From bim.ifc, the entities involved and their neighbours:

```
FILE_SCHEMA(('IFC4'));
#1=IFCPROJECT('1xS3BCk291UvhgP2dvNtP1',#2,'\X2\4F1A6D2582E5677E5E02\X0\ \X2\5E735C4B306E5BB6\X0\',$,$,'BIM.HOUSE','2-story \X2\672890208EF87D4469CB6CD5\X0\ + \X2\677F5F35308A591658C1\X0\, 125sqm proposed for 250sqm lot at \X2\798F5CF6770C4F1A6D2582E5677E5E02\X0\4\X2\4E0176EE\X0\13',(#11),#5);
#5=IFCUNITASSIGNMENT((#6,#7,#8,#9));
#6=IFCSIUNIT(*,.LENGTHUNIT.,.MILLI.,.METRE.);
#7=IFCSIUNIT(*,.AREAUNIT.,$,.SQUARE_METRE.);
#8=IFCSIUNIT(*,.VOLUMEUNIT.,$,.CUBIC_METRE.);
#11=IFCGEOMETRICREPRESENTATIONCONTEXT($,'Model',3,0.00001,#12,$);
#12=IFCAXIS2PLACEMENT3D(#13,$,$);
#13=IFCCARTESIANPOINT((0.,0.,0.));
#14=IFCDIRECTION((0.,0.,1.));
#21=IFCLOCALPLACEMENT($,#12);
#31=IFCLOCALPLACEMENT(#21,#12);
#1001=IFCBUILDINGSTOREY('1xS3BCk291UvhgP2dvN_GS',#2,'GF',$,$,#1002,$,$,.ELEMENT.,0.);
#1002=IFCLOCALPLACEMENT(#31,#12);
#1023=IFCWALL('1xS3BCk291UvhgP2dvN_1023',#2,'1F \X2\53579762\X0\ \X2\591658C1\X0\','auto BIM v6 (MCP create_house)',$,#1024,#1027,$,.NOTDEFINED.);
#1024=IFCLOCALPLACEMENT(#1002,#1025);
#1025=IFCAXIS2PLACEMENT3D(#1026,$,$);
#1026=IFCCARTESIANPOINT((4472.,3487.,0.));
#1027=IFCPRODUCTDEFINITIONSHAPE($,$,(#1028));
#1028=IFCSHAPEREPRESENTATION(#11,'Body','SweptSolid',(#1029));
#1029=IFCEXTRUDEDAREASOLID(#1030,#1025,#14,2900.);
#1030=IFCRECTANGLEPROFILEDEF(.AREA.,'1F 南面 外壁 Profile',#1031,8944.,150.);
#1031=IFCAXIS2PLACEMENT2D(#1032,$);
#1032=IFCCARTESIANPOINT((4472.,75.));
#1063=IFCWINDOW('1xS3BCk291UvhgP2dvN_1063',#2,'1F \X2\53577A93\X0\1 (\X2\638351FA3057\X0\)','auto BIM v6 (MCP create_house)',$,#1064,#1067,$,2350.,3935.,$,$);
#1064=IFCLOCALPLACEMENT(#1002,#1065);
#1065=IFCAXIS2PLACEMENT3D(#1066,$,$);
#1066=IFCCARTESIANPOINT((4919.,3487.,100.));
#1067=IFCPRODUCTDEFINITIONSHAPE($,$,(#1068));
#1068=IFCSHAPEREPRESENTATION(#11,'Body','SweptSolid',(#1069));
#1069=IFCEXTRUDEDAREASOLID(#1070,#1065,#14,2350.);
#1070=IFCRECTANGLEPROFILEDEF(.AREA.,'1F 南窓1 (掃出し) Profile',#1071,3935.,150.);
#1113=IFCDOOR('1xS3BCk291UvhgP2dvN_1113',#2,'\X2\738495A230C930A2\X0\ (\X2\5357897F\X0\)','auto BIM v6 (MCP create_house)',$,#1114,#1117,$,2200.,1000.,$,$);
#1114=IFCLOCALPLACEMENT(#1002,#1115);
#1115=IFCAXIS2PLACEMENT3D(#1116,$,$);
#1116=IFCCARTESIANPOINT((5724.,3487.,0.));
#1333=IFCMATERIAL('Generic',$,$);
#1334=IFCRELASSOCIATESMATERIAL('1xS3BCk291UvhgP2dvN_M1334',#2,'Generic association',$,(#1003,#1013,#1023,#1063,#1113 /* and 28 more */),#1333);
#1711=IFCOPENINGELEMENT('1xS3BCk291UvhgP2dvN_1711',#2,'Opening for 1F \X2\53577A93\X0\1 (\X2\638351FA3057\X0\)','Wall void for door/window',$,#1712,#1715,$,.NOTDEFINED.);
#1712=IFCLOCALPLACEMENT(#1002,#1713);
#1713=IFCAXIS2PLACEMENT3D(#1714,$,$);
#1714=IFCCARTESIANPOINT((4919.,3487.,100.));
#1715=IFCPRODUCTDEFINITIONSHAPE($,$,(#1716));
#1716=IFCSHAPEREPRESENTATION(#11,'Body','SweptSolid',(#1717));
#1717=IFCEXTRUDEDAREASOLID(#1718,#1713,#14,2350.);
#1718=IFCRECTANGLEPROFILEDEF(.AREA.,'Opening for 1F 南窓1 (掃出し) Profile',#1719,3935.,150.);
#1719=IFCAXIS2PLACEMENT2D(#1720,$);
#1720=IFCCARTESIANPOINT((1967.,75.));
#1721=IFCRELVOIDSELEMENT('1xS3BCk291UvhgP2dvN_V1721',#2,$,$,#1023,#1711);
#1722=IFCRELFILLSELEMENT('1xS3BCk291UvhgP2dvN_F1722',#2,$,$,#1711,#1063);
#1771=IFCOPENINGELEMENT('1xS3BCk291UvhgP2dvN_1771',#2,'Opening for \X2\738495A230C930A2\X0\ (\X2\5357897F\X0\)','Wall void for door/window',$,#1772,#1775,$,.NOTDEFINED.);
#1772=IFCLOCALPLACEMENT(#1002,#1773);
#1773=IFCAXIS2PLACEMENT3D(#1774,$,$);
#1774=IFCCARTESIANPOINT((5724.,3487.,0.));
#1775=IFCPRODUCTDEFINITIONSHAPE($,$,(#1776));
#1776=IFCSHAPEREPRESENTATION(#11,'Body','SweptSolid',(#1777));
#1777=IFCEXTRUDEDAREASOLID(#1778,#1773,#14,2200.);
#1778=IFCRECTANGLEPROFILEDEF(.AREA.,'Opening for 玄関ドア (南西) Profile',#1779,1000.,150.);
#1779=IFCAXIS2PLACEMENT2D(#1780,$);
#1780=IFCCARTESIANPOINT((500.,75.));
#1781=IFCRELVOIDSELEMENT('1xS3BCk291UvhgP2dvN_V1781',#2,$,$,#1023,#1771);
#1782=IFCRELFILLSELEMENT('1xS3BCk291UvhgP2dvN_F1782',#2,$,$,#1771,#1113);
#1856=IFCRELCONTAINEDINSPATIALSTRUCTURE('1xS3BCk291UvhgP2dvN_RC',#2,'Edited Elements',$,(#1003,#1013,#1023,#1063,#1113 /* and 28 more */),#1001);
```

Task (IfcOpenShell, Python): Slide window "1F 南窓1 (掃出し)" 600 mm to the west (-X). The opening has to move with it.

```python
import ifcopenshell
import ifcopenshell.api.geometry
import ifcopenshell.util.placement
import ifcopenshell.util.unit

model = ifcopenshell.open("bim.ifc")
unit_scale = ifcopenshell.util.unit.calculate_unit_scale(model)

window = model.by_id(1063)
opening = window.FillsVoids[0].RelatingOpeningElement
wall = opening.VoidsElements[0].RelatingBuildingElement

wall_matrix = ifcopenshell.util.placement.get_local_placement(wall.ObjectPlacement)
shift = wall_matrix[:3, 0] * -0.6 / unit_scale
before = ifcopenshell.util.placement.get_local_placement(window.ObjectPlacement)[:3, 3].copy()

# The window is not placed relative to its opening, so move both.
for product in (opening, window):
    matrix = ifcopenshell.util.placement.get_local_placement(product.ObjectPlacement)
    matrix[:3, 3] += shift
    ifcopenshell.api.geometry.edit_object_placement(model, product=product, matrix=matrix, is_si=False)

after = ifcopenshell.util.placement.get_local_placement(window.ObjectPlacement)[:3, 3]
print("window moved by", (after - before).round(3) + 0.0)

model.write("bim_rev.ifc")
```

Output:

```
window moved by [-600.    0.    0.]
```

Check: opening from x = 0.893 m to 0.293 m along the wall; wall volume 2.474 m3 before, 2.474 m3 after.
